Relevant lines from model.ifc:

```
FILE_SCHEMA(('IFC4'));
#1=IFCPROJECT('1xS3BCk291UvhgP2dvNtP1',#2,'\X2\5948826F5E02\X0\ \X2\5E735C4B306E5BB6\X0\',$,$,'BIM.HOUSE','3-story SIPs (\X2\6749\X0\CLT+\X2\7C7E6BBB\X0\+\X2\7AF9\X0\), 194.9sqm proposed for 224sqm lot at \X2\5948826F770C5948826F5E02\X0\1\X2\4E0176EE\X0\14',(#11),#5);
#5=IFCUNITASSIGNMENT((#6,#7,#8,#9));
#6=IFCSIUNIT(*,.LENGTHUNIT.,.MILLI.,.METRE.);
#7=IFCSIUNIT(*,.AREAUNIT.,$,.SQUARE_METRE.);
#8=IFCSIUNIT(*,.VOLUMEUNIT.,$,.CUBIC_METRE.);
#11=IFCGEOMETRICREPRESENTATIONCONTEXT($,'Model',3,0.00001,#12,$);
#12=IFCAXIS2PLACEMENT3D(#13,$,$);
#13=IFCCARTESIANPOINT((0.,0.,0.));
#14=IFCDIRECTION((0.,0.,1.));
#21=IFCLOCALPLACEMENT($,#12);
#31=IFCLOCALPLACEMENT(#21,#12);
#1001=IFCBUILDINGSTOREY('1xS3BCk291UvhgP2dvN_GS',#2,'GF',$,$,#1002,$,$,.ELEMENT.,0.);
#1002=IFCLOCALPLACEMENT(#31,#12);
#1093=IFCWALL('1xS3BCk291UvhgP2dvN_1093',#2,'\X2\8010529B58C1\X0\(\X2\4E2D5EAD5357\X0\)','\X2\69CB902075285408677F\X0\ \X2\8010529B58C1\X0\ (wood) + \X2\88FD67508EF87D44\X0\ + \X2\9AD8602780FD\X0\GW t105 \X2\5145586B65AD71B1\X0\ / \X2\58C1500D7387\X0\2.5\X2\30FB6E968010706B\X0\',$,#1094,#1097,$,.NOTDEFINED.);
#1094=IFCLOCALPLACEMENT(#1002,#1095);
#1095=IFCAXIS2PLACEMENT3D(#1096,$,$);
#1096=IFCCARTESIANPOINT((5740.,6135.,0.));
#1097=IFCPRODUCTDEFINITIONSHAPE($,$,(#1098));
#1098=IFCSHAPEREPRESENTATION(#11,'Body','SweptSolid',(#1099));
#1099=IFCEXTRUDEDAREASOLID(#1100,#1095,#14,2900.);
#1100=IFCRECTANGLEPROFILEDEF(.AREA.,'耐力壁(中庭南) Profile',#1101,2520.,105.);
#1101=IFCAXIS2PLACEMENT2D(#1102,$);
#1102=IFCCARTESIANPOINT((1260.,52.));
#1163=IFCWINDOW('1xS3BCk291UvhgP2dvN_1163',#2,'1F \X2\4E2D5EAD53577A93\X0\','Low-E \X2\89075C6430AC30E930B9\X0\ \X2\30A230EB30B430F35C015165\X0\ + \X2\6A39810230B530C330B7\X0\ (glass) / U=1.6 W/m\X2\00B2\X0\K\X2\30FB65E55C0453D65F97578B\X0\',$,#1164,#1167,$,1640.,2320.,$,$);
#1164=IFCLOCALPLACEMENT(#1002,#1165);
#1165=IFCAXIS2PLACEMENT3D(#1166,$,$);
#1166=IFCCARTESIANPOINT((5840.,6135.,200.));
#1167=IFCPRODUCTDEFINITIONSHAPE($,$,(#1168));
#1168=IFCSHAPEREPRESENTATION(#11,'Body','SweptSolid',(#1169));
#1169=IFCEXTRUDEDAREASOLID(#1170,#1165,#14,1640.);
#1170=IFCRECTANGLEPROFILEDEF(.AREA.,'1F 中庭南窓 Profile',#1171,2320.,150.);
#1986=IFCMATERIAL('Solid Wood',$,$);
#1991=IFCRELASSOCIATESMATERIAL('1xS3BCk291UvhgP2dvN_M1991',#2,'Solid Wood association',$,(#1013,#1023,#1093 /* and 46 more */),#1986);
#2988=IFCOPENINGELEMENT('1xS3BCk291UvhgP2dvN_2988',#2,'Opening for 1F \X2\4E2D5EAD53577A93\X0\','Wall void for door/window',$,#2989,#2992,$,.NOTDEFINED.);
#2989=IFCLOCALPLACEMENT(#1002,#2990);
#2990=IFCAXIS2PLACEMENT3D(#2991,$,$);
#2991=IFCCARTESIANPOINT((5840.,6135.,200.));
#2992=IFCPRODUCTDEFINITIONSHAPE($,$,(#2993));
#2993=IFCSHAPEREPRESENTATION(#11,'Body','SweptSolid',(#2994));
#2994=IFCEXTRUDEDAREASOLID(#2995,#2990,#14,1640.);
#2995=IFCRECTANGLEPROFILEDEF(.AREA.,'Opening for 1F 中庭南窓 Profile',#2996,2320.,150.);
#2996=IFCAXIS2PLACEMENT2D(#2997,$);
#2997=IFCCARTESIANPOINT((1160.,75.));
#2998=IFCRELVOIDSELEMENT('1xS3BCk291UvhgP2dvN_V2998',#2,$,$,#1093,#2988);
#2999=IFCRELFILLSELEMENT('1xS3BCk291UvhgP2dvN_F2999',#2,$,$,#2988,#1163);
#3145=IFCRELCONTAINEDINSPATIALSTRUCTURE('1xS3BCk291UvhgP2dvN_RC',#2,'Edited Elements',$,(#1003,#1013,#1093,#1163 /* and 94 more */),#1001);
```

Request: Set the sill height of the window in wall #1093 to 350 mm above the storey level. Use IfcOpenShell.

```python
import numpy as np
import ifcopenshell
import ifcopenshell.api.geometry
import ifcopenshell.geom
import ifcopenshell.util.element
import ifcopenshell.util.placement
import ifcopenshell.util.shape
import ifcopenshell.util.unit

model = ifcopenshell.open("model.ifc")
unit_scale = ifcopenshell.util.unit.calculate_unit_scale(model)

window = model.by_id(1163)
opening = window.FillsVoids[0].RelatingOpeningElement
storey = ifcopenshell.util.element.get_container(window, ifc_class="IfcBuildingStorey")
level = ifcopenshell.util.placement.get_local_placement(storey.ObjectPlacement)[2, 3]

# The opening's origin need not be at the sill, so measure its lowest point.
shape = ifcopenshell.geom.create_shape(ifcopenshell.geom.settings(), opening)
bottom = ifcopenshell.util.shape.get_shape_bottom_elevation(shape, shape.geometry) / unit_scale
dz = level + 0.35 / unit_scale - bottom

shift = np.array([0.0, 0.0, dz])
# The window is not placed relative to its opening, so move both.
for product in (opening, window):
    matrix = ifcopenshell.util.placement.get_local_placement(product.ObjectPlacement)
    matrix[:3, 3] += shift
    ifcopenshell.api.geometry.edit_object_placement(model, product=product, matrix=matrix, is_si=False)

print(f"moved by {dz * unit_scale:+.3f} m")

model.write("model_updated.ifc")
```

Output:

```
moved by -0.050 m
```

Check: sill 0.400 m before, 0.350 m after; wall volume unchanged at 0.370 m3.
